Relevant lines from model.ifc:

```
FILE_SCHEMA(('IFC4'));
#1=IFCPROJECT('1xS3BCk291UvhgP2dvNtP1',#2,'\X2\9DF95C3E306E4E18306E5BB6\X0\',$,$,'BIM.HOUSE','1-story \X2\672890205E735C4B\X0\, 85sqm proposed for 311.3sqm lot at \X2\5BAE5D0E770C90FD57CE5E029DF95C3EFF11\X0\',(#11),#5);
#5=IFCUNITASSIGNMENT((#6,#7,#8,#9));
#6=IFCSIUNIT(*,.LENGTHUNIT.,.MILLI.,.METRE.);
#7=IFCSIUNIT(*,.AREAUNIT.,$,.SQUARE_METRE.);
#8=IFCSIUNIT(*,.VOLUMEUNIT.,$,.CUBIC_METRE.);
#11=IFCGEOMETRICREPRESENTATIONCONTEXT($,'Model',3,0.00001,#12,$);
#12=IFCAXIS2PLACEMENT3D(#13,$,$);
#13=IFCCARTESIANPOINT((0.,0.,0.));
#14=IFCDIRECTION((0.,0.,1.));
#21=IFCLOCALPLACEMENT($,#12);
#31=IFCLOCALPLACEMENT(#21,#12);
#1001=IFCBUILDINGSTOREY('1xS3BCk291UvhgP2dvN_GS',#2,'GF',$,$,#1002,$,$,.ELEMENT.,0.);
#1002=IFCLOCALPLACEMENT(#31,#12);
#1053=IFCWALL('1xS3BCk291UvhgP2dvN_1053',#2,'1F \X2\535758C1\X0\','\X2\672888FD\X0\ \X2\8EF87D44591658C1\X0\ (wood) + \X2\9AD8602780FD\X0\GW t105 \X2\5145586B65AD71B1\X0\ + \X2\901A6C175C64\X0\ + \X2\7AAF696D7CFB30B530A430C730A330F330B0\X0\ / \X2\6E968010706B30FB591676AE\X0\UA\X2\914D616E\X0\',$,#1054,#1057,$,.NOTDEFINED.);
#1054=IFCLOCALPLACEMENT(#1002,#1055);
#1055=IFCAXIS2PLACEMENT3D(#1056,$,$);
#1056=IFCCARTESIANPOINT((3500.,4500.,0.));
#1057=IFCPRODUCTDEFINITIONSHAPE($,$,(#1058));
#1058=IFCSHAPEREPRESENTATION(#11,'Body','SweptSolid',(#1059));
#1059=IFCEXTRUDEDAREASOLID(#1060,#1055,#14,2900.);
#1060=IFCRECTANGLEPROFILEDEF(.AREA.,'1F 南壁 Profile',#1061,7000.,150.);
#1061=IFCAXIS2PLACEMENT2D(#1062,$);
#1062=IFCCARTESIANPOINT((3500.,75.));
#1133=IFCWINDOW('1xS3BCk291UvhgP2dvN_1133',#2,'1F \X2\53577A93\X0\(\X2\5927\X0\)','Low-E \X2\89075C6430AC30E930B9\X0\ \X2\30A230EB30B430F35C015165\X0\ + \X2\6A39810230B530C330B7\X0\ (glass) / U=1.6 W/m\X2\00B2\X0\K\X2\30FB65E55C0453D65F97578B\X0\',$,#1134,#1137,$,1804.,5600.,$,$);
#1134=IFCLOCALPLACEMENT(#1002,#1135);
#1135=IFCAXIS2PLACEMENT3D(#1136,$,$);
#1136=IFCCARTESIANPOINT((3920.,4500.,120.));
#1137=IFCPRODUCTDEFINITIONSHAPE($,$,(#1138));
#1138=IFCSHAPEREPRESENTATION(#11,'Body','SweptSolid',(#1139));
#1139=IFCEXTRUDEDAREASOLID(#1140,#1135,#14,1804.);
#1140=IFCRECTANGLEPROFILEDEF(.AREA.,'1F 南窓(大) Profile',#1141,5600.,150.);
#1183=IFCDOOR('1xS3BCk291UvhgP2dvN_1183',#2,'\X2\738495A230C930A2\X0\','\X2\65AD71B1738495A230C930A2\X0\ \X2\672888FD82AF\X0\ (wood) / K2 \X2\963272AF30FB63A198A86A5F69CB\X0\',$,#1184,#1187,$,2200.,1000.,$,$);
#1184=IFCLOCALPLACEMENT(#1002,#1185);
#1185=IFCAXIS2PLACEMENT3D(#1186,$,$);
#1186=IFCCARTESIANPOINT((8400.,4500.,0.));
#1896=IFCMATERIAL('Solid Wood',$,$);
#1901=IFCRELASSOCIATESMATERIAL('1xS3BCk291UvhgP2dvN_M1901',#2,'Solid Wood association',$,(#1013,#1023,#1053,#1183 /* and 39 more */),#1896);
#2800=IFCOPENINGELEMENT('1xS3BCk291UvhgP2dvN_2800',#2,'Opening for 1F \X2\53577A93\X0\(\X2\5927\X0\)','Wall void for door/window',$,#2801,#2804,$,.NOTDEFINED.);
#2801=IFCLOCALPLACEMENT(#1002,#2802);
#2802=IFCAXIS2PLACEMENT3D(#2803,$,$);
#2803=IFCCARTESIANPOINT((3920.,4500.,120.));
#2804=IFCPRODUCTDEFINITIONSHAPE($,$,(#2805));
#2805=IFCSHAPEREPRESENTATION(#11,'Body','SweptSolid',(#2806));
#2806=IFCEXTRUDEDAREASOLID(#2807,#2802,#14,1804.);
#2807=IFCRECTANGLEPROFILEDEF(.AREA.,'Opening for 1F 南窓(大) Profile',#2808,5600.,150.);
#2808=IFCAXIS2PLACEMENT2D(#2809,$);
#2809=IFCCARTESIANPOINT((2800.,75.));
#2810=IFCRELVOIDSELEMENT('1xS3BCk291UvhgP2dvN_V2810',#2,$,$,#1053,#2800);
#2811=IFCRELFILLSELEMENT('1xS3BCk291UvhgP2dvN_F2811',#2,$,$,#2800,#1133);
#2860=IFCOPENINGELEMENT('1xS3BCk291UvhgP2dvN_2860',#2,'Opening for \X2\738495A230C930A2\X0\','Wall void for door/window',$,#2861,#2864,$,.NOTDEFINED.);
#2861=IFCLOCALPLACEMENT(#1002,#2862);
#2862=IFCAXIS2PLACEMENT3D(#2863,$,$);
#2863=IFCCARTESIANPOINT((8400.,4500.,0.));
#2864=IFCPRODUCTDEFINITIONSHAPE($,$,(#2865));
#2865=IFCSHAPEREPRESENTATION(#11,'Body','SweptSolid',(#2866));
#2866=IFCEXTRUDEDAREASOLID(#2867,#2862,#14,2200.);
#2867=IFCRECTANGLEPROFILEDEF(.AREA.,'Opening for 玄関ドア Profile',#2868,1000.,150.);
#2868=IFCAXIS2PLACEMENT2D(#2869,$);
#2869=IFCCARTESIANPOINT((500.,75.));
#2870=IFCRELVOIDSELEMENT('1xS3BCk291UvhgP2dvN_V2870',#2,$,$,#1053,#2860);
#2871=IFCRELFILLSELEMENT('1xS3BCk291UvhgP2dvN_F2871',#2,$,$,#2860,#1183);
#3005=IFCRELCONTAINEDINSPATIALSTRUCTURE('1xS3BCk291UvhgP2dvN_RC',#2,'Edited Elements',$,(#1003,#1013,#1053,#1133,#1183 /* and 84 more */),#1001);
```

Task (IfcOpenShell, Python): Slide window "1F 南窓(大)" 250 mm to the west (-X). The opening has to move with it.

```python
import ifcopenshell
import ifcopenshell.api.geometry
import ifcopenshell.util.placement
import ifcopenshell.util.unit

model = ifcopenshell.open("model.ifc")
unit_scale = ifcopenshell.util.unit.calculate_unit_scale(model)

window = model.by_guid("1xS3BCk291UvhgP2dvN_1133")
opening = window.FillsVoids[0].RelatingOpeningElement
wall = opening.VoidsElements[0].RelatingBuildingElement

wall_matrix = ifcopenshell.util.placement.get_local_placement(wall.ObjectPlacement)
shift = wall_matrix[:3, 0] * -0.25 / unit_scale
before = ifcopenshell.util.placement.get_local_placement(window.ObjectPlacement)[:3, 3].copy()

# The window is not placed relative to its opening, so move both.
for product in (opening, window):
    matrix = ifcopenshell.util.placement.get_local_placement(product.ObjectPlacement)
    matrix[:3, 3] += shift
    ifcopenshell.api.geometry.edit_object_placement(model, product=product, matrix=matrix, is_si=False)

after = ifcopenshell.util.placement.get_local_placement(window.ObjectPlacement)[:3, 3]
print("window moved by", (after - before).round(3) + 0.0)

model.write("model_edited.ifc")
```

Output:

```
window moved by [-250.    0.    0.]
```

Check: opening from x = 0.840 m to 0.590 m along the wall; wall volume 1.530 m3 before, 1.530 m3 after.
